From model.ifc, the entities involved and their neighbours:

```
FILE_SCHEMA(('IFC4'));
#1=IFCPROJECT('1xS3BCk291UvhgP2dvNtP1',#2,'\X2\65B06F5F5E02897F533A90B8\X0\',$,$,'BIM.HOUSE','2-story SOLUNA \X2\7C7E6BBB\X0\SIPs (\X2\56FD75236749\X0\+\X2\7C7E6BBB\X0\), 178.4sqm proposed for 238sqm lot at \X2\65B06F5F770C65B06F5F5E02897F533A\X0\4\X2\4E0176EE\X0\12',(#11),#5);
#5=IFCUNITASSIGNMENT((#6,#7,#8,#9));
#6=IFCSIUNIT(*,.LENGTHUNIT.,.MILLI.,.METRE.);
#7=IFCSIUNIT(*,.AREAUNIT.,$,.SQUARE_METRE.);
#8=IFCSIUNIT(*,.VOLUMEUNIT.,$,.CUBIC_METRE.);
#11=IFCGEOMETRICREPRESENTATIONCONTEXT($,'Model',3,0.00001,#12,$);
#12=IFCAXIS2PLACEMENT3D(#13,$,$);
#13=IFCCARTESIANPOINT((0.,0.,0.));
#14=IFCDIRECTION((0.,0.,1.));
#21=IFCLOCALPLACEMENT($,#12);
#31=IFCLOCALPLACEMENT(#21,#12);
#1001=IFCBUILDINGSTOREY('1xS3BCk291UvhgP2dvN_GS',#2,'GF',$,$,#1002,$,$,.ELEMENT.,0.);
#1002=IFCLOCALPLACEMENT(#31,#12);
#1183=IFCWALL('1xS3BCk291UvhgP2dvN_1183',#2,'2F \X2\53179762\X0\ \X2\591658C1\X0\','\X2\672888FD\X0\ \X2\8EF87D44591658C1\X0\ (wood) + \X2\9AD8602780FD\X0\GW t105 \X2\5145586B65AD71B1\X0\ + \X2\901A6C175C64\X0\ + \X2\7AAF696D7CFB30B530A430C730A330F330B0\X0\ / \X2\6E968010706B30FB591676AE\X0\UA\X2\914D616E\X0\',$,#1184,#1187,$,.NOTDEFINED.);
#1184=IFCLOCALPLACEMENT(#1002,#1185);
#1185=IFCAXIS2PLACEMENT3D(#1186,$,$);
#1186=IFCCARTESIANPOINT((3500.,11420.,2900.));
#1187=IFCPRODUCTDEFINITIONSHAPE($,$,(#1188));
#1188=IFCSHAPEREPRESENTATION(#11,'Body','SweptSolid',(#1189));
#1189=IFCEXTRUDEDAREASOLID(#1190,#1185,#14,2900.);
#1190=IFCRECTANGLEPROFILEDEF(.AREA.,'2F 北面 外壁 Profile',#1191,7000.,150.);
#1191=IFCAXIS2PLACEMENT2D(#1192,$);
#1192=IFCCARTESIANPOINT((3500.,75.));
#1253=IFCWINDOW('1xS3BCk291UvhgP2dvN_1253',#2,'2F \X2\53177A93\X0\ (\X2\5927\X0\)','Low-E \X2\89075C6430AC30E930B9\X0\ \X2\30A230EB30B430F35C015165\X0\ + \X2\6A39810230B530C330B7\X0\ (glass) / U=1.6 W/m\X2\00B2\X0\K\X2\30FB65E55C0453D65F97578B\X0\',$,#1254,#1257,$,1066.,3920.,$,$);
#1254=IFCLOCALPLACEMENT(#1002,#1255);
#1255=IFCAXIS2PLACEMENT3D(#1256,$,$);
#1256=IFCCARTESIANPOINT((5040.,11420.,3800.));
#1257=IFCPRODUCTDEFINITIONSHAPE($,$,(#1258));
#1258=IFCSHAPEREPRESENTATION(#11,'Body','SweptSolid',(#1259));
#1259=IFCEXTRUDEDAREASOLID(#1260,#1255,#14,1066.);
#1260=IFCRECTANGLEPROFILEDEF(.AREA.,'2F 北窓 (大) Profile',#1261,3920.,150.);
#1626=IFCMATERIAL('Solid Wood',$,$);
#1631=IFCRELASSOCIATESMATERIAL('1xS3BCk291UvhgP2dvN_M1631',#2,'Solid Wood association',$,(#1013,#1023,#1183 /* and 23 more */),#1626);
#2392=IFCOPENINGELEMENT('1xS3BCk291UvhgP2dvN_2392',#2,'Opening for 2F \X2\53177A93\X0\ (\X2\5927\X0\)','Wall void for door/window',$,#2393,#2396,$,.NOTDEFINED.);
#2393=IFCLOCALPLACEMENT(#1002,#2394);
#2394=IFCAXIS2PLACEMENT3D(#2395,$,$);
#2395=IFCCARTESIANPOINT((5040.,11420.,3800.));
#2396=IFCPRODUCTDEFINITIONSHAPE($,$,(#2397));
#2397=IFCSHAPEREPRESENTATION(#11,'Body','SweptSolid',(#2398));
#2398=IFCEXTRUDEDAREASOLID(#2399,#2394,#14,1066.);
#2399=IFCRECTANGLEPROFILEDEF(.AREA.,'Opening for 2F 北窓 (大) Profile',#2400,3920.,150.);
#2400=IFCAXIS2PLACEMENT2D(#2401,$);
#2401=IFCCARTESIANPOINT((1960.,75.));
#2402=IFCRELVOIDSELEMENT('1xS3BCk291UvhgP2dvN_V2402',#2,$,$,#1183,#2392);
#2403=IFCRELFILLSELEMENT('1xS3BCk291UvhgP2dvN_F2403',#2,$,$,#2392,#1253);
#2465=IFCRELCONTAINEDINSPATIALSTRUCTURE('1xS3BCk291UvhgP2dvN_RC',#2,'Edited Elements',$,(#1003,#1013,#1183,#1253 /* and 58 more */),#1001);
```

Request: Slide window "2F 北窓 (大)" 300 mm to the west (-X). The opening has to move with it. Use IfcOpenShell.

```python
import ifcopenshell
import ifcopenshell.api.geometry
import ifcopenshell.util.placement

model = ifcopenshell.open("model.ifc")

window = model.by_guid("1xS3BCk291UvhgP2dvN_1253")
opening = window.FillsVoids[0].RelatingOpeningElement
wall = opening.VoidsElements[0].RelatingBuildingElement

wall_matrix = ifcopenshell.util.placement.get_local_placement(wall.ObjectPlacement)
shift = wall_matrix[:3, 0] * -300.0
before = ifcopenshell.util.placement.get_local_placement(window.ObjectPlacement)[:3, 3].copy()

# The window is not placed relative to its opening, so move both.
for product in (opening, window):
    matrix = ifcopenshell.util.placement.get_local_placement(product.ObjectPlacement)
    matrix[:3, 3] += shift
    ifcopenshell.api.geometry.edit_object_placement(model, product=product, matrix=matrix, is_si=False)

after = ifcopenshell.util.placement.get_local_placement(window.ObjectPlacement)[:3, 3]
print("window moved by", (after - before).round(3) + 0.0)

model.write("model-out.ifc")
```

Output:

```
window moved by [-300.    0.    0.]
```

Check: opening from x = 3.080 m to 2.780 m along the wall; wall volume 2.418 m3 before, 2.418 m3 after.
